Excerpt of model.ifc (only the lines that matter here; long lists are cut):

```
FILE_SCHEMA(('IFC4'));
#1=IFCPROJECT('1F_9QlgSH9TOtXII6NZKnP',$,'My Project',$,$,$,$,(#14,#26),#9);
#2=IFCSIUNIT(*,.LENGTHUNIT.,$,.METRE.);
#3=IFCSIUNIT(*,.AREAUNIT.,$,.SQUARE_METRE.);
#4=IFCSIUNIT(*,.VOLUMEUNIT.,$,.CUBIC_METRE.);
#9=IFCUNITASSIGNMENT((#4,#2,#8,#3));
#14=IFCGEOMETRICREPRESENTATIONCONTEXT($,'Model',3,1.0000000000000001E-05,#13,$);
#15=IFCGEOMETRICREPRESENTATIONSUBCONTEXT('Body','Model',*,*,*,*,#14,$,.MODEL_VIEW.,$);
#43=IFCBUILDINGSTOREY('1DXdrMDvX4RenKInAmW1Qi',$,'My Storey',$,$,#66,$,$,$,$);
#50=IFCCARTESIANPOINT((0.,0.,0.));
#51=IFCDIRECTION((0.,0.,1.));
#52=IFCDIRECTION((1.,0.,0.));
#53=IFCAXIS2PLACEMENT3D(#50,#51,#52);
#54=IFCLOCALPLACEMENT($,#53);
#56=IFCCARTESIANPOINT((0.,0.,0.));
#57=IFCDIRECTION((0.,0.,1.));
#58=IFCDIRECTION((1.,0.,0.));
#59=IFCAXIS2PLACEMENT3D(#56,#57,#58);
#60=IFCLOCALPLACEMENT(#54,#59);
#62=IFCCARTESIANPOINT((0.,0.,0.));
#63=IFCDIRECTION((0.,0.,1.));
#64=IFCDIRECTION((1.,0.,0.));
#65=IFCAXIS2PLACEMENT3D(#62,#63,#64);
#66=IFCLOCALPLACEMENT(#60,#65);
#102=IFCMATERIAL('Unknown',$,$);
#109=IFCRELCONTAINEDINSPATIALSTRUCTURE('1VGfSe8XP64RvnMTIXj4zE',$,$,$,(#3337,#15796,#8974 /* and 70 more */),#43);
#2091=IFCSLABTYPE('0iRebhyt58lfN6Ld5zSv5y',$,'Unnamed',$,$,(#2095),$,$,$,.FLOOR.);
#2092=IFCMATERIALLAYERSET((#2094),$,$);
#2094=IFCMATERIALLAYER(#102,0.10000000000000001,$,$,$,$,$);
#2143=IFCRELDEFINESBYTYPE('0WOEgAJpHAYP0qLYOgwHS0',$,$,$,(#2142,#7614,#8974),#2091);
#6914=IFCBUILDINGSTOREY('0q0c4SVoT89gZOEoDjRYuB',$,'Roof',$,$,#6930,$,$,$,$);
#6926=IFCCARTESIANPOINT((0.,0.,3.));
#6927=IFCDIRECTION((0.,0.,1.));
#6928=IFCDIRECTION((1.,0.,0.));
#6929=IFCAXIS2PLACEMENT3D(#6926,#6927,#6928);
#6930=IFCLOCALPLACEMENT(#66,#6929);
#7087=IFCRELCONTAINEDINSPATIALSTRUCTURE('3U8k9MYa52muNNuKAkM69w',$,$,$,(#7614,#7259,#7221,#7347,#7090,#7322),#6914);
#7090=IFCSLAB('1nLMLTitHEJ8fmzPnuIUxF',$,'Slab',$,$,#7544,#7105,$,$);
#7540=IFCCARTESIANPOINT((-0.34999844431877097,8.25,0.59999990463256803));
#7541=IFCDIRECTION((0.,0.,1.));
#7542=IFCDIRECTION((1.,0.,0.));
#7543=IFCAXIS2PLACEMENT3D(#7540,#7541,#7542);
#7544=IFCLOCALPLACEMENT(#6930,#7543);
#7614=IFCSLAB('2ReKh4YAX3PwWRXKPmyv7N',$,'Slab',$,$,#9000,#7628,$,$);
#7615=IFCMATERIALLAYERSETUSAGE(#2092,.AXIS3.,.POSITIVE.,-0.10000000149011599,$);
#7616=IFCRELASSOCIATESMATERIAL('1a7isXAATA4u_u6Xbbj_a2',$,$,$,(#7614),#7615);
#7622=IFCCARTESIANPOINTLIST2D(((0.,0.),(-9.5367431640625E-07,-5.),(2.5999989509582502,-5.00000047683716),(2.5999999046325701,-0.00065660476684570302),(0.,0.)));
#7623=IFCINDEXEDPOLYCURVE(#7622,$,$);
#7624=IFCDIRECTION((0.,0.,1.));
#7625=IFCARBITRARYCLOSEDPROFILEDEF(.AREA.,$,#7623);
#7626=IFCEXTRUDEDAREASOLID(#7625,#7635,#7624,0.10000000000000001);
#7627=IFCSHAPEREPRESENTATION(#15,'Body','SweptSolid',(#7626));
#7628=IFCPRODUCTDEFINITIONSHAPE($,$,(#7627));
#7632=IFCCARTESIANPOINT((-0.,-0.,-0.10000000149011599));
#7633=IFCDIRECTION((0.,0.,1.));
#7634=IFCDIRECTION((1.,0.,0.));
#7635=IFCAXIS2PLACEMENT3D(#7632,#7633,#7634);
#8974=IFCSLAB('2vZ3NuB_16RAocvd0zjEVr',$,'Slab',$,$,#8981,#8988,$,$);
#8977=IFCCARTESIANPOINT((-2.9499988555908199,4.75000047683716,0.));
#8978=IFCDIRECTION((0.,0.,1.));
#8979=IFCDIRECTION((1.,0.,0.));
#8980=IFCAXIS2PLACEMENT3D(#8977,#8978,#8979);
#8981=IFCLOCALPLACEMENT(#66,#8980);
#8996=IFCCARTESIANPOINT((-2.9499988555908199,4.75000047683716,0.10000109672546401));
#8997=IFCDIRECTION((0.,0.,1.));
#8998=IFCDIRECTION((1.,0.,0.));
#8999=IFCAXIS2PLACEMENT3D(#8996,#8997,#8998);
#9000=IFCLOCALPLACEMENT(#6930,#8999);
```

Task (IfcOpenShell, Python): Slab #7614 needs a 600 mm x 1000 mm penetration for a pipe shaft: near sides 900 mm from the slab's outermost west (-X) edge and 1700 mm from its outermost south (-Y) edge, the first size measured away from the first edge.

```python
import numpy as np
import ifcopenshell
import ifcopenshell.api.feature
import ifcopenshell.api.geometry
import ifcopenshell.api.root
import ifcopenshell.geom
import ifcopenshell.util.placement
import ifcopenshell.util.representation
import ifcopenshell.util.shape
import ifcopenshell.util.unit

model = ifcopenshell.open("model.ifc")
unit_scale = ifcopenshell.util.unit.calculate_unit_scale(model)
settings = ifcopenshell.geom.settings()


def volume(element):
    """Net volume in cubic metres, openings subtracted."""
    shape = ifcopenshell.geom.create_shape(settings, element)
    return ifcopenshell.util.shape.get_volume(shape.geometry)


slab = model.by_guid("2ReKh4YAX3PwWRXKPmyv7N")
before = volume(slab)

# Extent in the slab's own axes, in metres. The edges named are its -X and -Y sides.
slab_shape = ifcopenshell.geom.create_shape(settings, slab)
vertices = ifcopenshell.util.shape.get_vertices(slab_shape.geometry)
x_min, y_min, bottom = vertices.min(axis=0)
top = vertices[:, 2].max()

opening = ifcopenshell.api.root.create_entity(model, ifc_class="IfcOpeningElement", name="Pipe shaft opening", predefined_type="OPENING")
context = ifcopenshell.util.representation.get_context(model, "Model", "Body", "MODEL_VIEW")
width, depth = 0.6, 1
outline = [(0.0, 0.0), (width, 0.0), (width, depth), (0.0, depth), (0.0, 0.0)]
# Overshoot both faces by 50 mm so the cut is clean.
shape = ifcopenshell.api.geometry.add_slab_representation(
    model, context=context, depth=top - bottom + 0.1, polyline=outline
)
ifcopenshell.api.geometry.assign_representation(model, product=opening, representation=shape)

matrix = ifcopenshell.util.placement.get_local_placement(slab.ObjectPlacement)
matrix[:, 3] = matrix @ np.append(np.array([x_min + 0.9, y_min + 1.7, bottom - 0.05]) / unit_scale, 1.0)
ifcopenshell.api.geometry.edit_object_placement(model, product=opening, matrix=matrix, is_si=False)
ifcopenshell.api.feature.add_feature(model, feature=opening, element=slab)

after = volume(slab)

print(f"slab volume {before:.3f} -> {after:.3f} m3")

model.write("model_rev.ifc")
```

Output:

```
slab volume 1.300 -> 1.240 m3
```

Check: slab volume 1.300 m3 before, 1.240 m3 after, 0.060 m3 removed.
